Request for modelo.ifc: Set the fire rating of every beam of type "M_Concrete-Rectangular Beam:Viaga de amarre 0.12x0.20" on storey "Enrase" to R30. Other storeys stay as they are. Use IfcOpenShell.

First a look at what the model holds.

```python
import ifcopenshell
import ifcopenshell.util.element

model = ifcopenshell.open("modelo.ifc")
print(model.schema)
storey = next(s for s in model.by_type("IfcBuildingStorey") if s.Name == "Enrase")
beams = [e for e in ifcopenshell.util.element.get_decomposition(storey) if e.is_a("IfcBeam")]
seen = {}
for e in beams:
    element_type = ifcopenshell.util.element.get_type(e)
    key = (element_type.Name if element_type != e and element_type else None, ifcopenshell.util.element.get_pset(e, "Pset_BeamCommon", "FireRating"))
    seen[key] = seen.get(key, 0) + 1
for (name, value), count in sorted(seen.items(), key=str):
    print(count, "x", name, "|", value)
```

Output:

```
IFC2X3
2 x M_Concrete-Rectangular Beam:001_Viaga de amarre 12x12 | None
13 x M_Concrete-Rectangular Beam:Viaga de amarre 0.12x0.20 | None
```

```python
import ifcopenshell
import ifcopenshell.api.pset
import ifcopenshell.util.element

model = ifcopenshell.open("modelo.ifc")

storey = next(s for s in model.by_type("IfcBuildingStorey") if s.Name == "Enrase")
beams = [e for e in ifcopenshell.util.element.get_decomposition(storey) if e.is_a("IfcBeam")]

count = 0
for e in beams:
    element_type = ifcopenshell.util.element.get_type(e)
    if element_type in (None, e) or element_type.Name != "M_Concrete-Rectangular Beam:Viaga de amarre 0.12x0.20":
        continue
    # add_pset returns the element's existing set when there is one.
    pset = ifcopenshell.api.pset.add_pset(model, product=e, name="Pset_BeamCommon")
    ifcopenshell.api.pset.edit_pset(model, pset=pset, properties={"FireRating": "R30"})
    count += 1

print(count, "beams updated")

model.write("modelo_edited.ifc")
```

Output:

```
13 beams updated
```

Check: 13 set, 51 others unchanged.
